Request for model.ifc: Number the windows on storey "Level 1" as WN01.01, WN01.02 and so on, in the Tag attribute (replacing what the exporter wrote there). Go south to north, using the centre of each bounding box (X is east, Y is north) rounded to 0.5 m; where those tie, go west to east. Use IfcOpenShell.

First a look at what the model holds.

```python
import ifcopenshell
import ifcopenshell.util.element
import ifcopenshell.util.placement

model = ifcopenshell.open("model.ifc")
print(model.schema)
storey = next(s for s in model.by_type("IfcBuildingStorey") if s.Name == "Level 1")
windows = [e for e in ifcopenshell.util.element.get_decomposition(storey) if e.is_a("IfcWindow")]
for e in sorted(windows, key=lambda e: e.id()):
    origin = ifcopenshell.util.placement.get_local_placement(e.ObjectPlacement)[:3, 3]
    print(e.id(), e.Tag, e.Name, origin.round(2) + 0.0, sep=" | ")
```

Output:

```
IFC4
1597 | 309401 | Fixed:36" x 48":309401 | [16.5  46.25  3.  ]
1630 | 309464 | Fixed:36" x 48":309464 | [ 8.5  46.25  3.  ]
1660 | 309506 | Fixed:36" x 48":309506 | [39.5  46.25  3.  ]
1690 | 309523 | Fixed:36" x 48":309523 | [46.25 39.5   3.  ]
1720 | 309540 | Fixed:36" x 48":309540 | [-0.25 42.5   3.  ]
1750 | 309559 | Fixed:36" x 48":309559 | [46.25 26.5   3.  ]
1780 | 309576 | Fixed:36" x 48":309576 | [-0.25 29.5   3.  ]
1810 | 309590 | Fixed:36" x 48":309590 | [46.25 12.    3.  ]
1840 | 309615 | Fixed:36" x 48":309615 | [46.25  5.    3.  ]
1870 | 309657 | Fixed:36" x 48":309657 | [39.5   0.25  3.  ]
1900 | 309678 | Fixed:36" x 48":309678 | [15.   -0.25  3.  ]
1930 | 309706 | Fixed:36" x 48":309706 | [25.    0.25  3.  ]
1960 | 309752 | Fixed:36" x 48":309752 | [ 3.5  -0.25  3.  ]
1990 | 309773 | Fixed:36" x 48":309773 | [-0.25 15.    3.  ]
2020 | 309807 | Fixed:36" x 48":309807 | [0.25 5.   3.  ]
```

```python
import ifcopenshell
import ifcopenshell.geom
import ifcopenshell.util.element
import ifcopenshell.util.shape

model = ifcopenshell.open("model.ifc")
settings = ifcopenshell.geom.settings()
settings.set("use-world-coords", True)


def centre(element):
    shape = ifcopenshell.geom.create_shape(settings, element)
    return ifcopenshell.util.shape.get_bbox_centroid(shape.geometry)


storey = next(s for s in model.by_type("IfcBuildingStorey") if s.Name == "Level 1")
windows = [e for e in ifcopenshell.util.element.get_decomposition(storey) if e.is_a("IfcWindow")]

# Insertion points can sit at a corner or the storey origin, so sort by the geometry (in metres).
centres = {e: centre(e) for e in windows}
windows.sort(key=lambda e: (round(centres[e][1] / 0.5), centres[e][0]))

for i, e in enumerate(windows, start=1):
    number = f"WN01.{i:02d}"
    e.Tag = number
    print(e.id(), number)

model.write("model_edited.ifc")
```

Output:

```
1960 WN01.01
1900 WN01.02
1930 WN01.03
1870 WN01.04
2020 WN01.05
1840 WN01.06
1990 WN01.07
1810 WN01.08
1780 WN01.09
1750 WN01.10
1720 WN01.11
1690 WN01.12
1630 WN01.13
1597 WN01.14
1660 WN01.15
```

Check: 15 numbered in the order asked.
